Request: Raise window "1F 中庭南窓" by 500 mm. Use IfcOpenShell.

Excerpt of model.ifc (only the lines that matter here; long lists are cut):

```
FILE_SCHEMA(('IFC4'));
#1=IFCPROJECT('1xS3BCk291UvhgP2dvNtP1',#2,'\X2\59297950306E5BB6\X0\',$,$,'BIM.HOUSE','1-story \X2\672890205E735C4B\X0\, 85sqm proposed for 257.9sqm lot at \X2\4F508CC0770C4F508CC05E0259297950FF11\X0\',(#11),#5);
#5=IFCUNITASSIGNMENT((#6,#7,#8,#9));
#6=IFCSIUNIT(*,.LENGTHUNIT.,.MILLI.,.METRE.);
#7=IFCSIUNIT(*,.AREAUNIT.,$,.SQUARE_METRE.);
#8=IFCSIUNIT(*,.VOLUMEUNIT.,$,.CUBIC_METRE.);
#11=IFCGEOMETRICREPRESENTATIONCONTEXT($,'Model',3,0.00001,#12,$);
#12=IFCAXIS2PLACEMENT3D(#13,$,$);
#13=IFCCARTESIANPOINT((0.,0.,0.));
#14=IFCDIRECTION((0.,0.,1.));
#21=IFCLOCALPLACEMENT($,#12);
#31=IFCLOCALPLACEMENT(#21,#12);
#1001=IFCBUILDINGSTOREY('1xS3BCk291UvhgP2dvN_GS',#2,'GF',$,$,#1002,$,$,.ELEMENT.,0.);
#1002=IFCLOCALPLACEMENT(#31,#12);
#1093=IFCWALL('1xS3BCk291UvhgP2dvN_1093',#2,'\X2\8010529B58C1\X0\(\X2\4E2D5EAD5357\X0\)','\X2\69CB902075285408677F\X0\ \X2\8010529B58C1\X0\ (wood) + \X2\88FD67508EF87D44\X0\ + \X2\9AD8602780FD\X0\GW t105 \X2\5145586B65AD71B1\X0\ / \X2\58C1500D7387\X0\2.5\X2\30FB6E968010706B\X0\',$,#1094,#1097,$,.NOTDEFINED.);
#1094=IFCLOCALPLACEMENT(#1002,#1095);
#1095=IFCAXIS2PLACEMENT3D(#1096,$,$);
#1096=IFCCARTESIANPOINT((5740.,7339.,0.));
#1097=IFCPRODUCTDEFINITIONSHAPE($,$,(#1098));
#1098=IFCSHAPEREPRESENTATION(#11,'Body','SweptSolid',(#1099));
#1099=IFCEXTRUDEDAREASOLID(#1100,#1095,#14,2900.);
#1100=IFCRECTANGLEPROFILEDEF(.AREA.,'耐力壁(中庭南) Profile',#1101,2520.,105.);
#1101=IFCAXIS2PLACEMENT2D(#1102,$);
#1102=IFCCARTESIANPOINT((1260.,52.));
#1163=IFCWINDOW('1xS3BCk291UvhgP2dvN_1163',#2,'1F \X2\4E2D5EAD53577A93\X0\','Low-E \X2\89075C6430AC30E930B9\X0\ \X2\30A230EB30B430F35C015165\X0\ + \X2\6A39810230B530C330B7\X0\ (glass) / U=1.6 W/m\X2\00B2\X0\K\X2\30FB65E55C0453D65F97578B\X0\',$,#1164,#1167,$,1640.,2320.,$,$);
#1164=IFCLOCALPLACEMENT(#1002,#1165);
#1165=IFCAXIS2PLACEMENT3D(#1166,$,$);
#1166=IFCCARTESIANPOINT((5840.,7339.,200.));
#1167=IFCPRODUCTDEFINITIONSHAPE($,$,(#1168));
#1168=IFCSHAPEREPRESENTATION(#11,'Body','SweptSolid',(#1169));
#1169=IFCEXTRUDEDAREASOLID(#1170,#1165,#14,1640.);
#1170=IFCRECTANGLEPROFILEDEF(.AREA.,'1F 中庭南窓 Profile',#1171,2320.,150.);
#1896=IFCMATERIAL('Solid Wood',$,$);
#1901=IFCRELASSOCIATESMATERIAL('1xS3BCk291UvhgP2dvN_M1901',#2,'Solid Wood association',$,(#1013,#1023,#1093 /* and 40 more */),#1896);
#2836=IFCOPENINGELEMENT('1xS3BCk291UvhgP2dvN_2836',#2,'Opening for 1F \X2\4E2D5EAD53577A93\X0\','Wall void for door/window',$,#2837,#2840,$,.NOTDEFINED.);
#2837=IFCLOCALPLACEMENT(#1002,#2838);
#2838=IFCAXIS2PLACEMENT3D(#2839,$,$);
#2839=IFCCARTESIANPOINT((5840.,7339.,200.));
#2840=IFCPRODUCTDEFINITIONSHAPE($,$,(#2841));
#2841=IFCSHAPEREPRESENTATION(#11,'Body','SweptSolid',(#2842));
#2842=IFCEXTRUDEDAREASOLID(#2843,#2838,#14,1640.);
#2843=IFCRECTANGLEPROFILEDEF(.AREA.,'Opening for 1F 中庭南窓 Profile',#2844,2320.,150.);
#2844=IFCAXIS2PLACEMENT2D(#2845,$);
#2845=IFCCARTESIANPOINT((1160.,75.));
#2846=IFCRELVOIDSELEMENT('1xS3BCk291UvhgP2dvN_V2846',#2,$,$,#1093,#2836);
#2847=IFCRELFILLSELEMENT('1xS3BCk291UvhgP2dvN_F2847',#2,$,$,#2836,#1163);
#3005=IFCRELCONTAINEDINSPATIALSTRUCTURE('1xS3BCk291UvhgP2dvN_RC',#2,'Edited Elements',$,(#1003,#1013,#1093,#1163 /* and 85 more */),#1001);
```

```python
import numpy as np
import ifcopenshell
import ifcopenshell.api.geometry
import ifcopenshell.util.placement
import ifcopenshell.util.unit

model = ifcopenshell.open("model.ifc")
unit_scale = ifcopenshell.util.unit.calculate_unit_scale(model)

window = model.by_guid("1xS3BCk291UvhgP2dvN_1163")
opening = window.FillsVoids[0].RelatingOpeningElement
dz = 500.0

shift = np.array([0.0, 0.0, dz])
# The window is not placed relative to its opening, so move both.
for product in (opening, window):
    matrix = ifcopenshell.util.placement.get_local_placement(product.ObjectPlacement)
    matrix[:3, 3] += shift
    ifcopenshell.api.geometry.edit_object_placement(model, product=product, matrix=matrix, is_si=False)

print(f"moved by {dz * unit_scale:+.3f} m")

model.write("model-out.ifc")
```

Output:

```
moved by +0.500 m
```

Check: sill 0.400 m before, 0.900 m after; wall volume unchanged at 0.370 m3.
